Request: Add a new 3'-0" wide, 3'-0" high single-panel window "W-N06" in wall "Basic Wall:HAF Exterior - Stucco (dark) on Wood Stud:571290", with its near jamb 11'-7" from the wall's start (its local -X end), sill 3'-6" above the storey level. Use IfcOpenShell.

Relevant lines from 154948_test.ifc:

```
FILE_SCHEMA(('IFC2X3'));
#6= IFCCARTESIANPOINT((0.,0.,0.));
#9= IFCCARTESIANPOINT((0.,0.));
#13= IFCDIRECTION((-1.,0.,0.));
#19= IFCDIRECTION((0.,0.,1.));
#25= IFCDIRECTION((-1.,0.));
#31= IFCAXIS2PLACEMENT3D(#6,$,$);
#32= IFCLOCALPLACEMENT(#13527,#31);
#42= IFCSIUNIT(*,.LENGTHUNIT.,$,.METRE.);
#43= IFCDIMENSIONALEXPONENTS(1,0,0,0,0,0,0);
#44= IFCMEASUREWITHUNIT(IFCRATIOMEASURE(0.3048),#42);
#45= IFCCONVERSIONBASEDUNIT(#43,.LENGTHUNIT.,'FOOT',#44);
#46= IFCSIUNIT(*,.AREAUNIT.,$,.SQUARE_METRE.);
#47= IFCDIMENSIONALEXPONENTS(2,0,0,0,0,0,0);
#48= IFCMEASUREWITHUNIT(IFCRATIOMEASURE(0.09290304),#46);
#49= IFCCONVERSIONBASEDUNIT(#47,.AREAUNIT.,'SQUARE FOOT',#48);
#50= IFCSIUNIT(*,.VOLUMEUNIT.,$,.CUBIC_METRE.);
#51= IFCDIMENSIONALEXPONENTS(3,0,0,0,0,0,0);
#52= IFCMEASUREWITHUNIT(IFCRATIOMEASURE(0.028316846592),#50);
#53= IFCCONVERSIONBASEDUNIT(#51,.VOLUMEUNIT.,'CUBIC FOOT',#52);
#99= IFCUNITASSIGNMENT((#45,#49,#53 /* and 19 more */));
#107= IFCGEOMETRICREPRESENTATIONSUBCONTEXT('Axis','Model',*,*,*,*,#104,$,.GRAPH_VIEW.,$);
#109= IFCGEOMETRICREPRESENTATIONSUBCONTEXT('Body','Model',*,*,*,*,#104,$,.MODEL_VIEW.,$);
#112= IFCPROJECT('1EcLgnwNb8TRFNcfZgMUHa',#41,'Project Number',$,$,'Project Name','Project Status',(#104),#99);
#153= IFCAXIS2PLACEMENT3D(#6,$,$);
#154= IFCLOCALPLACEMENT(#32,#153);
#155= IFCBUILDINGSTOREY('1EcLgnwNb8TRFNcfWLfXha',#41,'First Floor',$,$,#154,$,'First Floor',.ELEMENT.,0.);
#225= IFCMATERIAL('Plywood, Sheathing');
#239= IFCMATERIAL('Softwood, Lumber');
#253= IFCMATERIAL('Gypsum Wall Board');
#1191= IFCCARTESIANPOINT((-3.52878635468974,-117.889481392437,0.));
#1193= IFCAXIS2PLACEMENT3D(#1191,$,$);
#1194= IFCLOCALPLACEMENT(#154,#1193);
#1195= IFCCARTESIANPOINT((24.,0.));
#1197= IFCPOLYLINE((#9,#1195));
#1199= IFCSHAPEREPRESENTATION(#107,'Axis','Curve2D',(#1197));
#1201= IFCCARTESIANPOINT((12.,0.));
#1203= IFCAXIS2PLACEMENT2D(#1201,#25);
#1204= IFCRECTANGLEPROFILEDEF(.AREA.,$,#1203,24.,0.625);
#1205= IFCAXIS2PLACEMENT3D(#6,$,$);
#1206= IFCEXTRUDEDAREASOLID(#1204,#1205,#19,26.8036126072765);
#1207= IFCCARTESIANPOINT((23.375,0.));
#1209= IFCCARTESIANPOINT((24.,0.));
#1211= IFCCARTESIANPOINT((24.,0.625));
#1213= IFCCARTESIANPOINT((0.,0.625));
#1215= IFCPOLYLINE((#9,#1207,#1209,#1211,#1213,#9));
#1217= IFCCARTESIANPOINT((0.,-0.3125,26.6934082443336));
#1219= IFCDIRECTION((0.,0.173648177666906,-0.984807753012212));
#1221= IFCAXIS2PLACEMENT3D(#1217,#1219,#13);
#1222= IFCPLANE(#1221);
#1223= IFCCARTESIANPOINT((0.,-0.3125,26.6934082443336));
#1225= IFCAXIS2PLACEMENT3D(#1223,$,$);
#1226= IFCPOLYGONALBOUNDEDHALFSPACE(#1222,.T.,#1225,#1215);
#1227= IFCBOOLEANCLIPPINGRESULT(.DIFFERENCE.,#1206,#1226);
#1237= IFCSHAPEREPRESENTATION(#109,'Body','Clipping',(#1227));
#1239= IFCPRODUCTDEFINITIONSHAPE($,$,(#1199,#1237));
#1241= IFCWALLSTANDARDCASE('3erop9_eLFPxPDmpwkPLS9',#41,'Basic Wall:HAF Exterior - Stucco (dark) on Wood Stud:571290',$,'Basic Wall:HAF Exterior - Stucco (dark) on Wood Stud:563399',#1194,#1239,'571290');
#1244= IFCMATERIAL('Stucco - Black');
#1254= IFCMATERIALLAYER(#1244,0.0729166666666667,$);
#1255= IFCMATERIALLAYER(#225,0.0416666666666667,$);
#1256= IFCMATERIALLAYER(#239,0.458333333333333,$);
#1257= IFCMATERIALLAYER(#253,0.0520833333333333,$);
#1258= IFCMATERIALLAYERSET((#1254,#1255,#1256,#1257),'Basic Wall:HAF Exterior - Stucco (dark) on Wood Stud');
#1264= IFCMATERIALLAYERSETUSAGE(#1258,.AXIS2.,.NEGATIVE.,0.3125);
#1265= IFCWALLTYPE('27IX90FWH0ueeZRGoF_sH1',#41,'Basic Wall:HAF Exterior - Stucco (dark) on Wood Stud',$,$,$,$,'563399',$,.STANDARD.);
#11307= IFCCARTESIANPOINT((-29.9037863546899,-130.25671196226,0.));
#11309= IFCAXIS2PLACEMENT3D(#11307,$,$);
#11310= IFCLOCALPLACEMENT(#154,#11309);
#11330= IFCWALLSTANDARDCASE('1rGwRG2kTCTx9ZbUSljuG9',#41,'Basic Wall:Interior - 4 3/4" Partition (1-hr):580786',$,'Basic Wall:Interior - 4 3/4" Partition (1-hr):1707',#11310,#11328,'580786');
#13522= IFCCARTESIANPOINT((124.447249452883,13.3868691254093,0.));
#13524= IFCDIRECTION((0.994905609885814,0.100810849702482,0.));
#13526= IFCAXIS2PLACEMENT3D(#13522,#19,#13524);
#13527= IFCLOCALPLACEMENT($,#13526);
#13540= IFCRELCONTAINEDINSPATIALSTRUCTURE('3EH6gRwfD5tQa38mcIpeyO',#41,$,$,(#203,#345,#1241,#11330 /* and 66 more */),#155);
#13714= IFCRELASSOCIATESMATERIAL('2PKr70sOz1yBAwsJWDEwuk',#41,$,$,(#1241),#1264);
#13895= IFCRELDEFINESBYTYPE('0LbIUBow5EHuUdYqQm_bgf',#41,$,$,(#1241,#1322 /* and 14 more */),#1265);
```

```python
import numpy as np
import ifcopenshell
import ifcopenshell.api.feature
import ifcopenshell.api.geometry
import ifcopenshell.api.root
import ifcopenshell.api.spatial
import ifcopenshell.api.type
import ifcopenshell.geom
import ifcopenshell.util.element
import ifcopenshell.util.placement
import ifcopenshell.util.representation
import ifcopenshell.util.shape
import ifcopenshell.util.unit

model = ifcopenshell.open("154948_test.ifc")
unit_scale = ifcopenshell.util.unit.calculate_unit_scale(model)
settings = ifcopenshell.geom.settings()


def volume(element):
    """Net volume in cubic metres, openings subtracted."""
    shape = ifcopenshell.geom.create_shape(settings, element)
    return ifcopenshell.util.shape.get_volume(shape.geometry)


wall = model.by_guid("3erop9_eLFPxPDmpwkPLS9")
storey = ifcopenshell.util.element.get_container(wall, ifc_class="IfcBuildingStorey")
context = ifcopenshell.util.representation.get_context(model, "Model", "Body", "MODEL_VIEW")
before = volume(wall)

width, height, from_end, sill = 0.9144, 0.9144, 3.5306, 1.0668  # metres

# The wall runs along its own X axis, and the end named is its -X end.
wall_shape = ifcopenshell.geom.create_shape(settings, wall)
x, y, z = ifcopenshell.util.shape.get_vertices(wall_shape.geometry).T
start = x.min() + from_end
face, thickness = float(y.min()), float(y.max() - y.min())
wall_matrix = ifcopenshell.util.placement.get_local_placement(wall.ObjectPlacement)
level = ifcopenshell.util.placement.get_local_placement(storey.ObjectPlacement)[2, 3]


def in_wall(x, y):
    """Placement at x, y metres in the wall's axes, at sill height."""
    matrix = wall_matrix.copy()
    matrix[:, 3] = wall_matrix @ np.array([x / unit_scale, y / unit_scale, 0.0, 1.0])
    matrix[2, 3] = level + sill / unit_scale
    return matrix


# Opening: a box that overshoots both wall faces by 50 mm.
opening = ifcopenshell.api.root.create_entity(model, ifc_class="IfcOpeningElement")
box = ifcopenshell.api.geometry.add_wall_representation(
    model, context=context, length=width, height=height, thickness=thickness + 0.1
)
ifcopenshell.api.geometry.assign_representation(model, product=opening, representation=box)
ifcopenshell.api.geometry.edit_object_placement(model, product=opening, matrix=in_wall(start, face - 0.05), is_si=False)
ifcopenshell.api.feature.add_feature(model, feature=opening, element=wall)

window = ifcopenshell.api.root.create_entity(model, ifc_class="IfcWindow", name="W-N06")
window.OverallWidth, window.OverallHeight = width / unit_scale, height / unit_scale
body = ifcopenshell.api.geometry.add_window_representation(
    model,
    context=context,
    overall_width=window.OverallWidth,
    overall_height=window.OverallHeight,
    partition_type="SINGLE_PANEL",
)
ifcopenshell.api.geometry.assign_representation(model, product=window, representation=body)
ifcopenshell.api.spatial.assign_container(model, products=[window], relating_structure=storey)
fills = ifcopenshell.api.feature.add_filling(model, opening=opening, element=window)
fills.OwnerHistory = window.OwnerHistory  # required in IFC2X3

# IFC2X3 keeps the operation on the window style.
style = ifcopenshell.api.root.create_entity(model, ifc_class="IfcWindowStyle", name="W-N06")
style.OperationType, style.ConstructionType = "SINGLE_PANEL", "NOTDEFINED"
style.ParameterTakesPrecedence = style.Sizeable = False
ifcopenshell.api.type.assign_type(model, related_objects=[window], relating_type=style)

# Centre the window in the wall's thickness.
ifcopenshell.api.geometry.edit_object_placement(model, product=window, matrix=in_wall(start, face), is_si=False)
window_shape = ifcopenshell.geom.create_shape(settings, window)
depth = ifcopenshell.util.shape.get_vertices(window_shape.geometry)[:, 1]
offset = face + thickness / 2 - (depth.min() + depth.max()) / 2
ifcopenshell.api.geometry.edit_object_placement(model, product=window, matrix=in_wall(start, offset), is_si=False)

after = volume(wall)

print(f"wall volume {before:.3f} -> {after:.3f} m3")

model.write("154948_test_edited.ifc")
```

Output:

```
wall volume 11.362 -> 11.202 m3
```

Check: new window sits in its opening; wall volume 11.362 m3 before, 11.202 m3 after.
